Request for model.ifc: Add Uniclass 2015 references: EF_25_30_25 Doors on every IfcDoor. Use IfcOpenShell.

First a look at what the model holds.

```python
import ifcopenshell

model = ifcopenshell.open("model.ifc")
print(model.schema)
print("classifications:", [c.Name for c in model.by_type("IfcClassification")])
for ifc_class in ("IfcDoor", "IfcRoof", "IfcStair", "IfcWall", "IfcWindow"):
    print(ifc_class, len(model.by_type(ifc_class)))
```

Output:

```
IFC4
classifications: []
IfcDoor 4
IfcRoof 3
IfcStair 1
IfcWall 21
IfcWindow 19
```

```python
import ifcopenshell
import ifcopenshell.api.classification

model = ifcopenshell.open("model.ifc")

system = ifcopenshell.api.classification.add_classification(model, classification="Uniclass 2015")

codes = {
    "IfcDoor": ("EF_25_30_25", "Doors"),
}
for ifc_class, (code, name) in codes.items():
    products = model.by_type(ifc_class)
    ifcopenshell.api.classification.add_reference(
        model, products=products, classification=system, identification=code, name=name
    )
    print(code, len(products))

model.write("model-out.ifc")
```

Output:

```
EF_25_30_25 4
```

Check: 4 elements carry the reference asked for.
